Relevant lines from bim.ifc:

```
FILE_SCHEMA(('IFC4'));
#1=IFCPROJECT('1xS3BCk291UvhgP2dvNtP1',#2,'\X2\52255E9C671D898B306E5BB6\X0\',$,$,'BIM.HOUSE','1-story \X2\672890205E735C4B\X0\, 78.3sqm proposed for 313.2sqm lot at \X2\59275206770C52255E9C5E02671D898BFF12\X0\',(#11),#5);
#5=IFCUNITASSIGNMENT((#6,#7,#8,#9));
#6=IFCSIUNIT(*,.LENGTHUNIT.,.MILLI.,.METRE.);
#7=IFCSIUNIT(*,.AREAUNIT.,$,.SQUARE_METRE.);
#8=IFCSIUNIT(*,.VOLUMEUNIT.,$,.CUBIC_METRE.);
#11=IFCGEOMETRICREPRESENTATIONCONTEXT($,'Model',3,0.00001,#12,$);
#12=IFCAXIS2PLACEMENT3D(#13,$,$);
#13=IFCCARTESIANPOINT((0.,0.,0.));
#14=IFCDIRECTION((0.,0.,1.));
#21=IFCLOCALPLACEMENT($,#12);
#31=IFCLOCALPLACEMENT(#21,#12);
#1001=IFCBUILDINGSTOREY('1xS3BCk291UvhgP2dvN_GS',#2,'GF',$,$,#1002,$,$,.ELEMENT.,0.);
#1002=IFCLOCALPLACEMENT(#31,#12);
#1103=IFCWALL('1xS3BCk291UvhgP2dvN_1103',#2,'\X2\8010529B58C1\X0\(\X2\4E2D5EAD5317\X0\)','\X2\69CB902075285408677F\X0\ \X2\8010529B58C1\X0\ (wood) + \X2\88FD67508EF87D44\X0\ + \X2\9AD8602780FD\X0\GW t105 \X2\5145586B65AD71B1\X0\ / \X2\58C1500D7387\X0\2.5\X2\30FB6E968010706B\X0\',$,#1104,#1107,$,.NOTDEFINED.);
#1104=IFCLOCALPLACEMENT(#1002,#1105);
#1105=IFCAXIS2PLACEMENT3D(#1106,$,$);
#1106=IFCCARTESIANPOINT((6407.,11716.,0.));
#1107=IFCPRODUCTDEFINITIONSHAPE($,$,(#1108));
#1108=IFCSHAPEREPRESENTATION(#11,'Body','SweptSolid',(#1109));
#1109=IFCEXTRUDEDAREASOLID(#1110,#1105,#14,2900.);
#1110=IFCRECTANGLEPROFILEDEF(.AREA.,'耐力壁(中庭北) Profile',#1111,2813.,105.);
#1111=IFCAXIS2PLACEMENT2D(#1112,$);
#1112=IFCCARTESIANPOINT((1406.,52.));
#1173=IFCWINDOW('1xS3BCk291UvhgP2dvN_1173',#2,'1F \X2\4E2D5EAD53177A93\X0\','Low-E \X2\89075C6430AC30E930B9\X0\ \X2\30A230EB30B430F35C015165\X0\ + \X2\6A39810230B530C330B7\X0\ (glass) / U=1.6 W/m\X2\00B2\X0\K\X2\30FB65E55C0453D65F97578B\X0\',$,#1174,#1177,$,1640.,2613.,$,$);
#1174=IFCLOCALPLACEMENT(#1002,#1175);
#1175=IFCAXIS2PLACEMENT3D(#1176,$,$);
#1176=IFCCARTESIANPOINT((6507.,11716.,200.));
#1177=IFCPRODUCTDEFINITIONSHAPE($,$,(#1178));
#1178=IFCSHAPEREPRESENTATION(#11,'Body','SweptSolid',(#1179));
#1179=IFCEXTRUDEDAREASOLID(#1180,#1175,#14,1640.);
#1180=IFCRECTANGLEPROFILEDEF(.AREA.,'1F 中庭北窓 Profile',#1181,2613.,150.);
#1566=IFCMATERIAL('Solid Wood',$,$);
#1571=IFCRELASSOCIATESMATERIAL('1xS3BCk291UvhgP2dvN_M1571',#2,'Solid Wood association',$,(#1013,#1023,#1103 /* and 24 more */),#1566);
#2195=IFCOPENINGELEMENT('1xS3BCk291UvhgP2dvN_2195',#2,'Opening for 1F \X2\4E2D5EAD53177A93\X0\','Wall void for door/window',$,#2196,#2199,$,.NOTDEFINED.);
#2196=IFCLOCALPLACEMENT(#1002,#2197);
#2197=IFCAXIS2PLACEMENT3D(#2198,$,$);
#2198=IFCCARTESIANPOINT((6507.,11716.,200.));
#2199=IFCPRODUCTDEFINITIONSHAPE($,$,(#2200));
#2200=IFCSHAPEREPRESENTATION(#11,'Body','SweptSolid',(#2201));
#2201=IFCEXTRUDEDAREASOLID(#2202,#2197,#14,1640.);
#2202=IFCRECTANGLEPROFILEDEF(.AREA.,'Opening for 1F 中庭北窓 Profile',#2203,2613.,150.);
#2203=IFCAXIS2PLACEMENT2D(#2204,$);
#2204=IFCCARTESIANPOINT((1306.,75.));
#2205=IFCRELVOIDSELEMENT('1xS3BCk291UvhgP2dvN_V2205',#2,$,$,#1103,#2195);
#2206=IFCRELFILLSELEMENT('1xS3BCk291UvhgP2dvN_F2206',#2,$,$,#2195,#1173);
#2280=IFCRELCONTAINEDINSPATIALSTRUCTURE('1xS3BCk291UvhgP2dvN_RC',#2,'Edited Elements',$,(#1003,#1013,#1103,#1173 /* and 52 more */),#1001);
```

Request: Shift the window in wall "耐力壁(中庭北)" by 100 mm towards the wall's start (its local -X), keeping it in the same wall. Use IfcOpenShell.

```python
import ifcopenshell
import ifcopenshell.api.geometry
import ifcopenshell.util.placement

model = ifcopenshell.open("bim.ifc")

window = model.by_guid("1xS3BCk291UvhgP2dvN_1173")
opening = window.FillsVoids[0].RelatingOpeningElement
wall = opening.VoidsElements[0].RelatingBuildingElement

wall_matrix = ifcopenshell.util.placement.get_local_placement(wall.ObjectPlacement)
shift = wall_matrix[:3, 0] * -100.0
before = ifcopenshell.util.placement.get_local_placement(window.ObjectPlacement)[:3, 3].copy()

# The window is not placed relative to its opening, so move both.
for product in (opening, window):
    matrix = ifcopenshell.util.placement.get_local_placement(product.ObjectPlacement)
    matrix[:3, 3] += shift
    ifcopenshell.api.geometry.edit_object_placement(model, product=product, matrix=matrix, is_si=False)

after = ifcopenshell.util.placement.get_local_placement(window.ObjectPlacement)[:3, 3]
print("window moved by", (after - before).round(3) + 0.0)

model.write("bim_edited.ifc")
```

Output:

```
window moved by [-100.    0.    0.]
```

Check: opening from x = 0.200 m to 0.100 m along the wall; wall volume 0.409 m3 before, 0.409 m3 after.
